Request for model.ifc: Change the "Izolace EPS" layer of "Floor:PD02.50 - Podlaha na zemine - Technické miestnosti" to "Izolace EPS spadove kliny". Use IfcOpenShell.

First a look at what the model holds.

```python
import ifcopenshell
import ifcopenshell.util.element

model = ifcopenshell.open("model.ifc")
print(model.schema)
for layer_set in model.by_type("IfcMaterialLayerSet"):
    if layer_set.LayerSetName == "Floor:PD02.50 - Podlaha na zemine - Technické miestnosti":
        for layer in layer_set.MaterialLayers:
            print(layer.id(), layer.Material and layer.Material.Name, layer.LayerThickness, sep=" | ")
        print(len(ifcopenshell.util.element.get_elements_by_material(model, layer_set)), "elements and types use it")
print(sorted(m.Name for m in model.by_type("IfcMaterial") if m.Name)[:60])
```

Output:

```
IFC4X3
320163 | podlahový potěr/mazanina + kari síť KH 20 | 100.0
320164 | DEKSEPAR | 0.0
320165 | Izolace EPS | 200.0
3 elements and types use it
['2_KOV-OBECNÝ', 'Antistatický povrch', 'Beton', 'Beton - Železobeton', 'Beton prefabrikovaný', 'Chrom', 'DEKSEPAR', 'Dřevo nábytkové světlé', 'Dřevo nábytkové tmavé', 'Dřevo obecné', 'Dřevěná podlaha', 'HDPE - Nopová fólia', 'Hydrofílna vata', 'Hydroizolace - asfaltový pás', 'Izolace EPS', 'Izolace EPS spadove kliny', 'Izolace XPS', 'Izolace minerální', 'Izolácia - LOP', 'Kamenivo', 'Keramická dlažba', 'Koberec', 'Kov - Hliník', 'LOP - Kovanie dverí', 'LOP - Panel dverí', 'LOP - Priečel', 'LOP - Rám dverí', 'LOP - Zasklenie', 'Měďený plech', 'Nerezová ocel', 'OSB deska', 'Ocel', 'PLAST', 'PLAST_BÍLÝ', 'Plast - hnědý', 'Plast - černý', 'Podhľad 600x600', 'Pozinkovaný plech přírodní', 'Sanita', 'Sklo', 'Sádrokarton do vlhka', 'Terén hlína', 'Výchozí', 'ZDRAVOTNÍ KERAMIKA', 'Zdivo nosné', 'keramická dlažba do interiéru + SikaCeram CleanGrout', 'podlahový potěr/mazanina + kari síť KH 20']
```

```python
import ifcopenshell
import ifcopenshell.api.material

model = ifcopenshell.open("model.ifc")

layer_set = next(s for s in model.by_type("IfcMaterialLayerSet") if s.LayerSetName == "Floor:PD02.50 - Podlaha na zemine - Technické miestnosti")
layer = next(l for l in layer_set.MaterialLayers if l.Material and l.Material.Name == "Izolace EPS")
material = next(m for m in model.by_type("IfcMaterial") if m.Name == "Izolace EPS spadove kliny")

# Point this one layer at the other material; renaming the old one would change it everywhere.
ifcopenshell.api.material.edit_layer(model, layer=layer, attributes={"Name": material.Name}, material=material)

print([l.Material.Name if l.Material else None for l in layer_set.MaterialLayers])

model.write("model_rev.ifc")
```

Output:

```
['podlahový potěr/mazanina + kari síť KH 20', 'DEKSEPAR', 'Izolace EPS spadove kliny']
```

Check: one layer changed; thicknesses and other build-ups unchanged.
